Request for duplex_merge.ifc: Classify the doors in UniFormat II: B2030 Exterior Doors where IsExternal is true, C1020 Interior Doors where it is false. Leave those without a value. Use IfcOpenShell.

First a look at what the model holds.

```python
import ifcopenshell
import ifcopenshell.util.element

model = ifcopenshell.open("duplex_merge.ifc")
print(model.schema)
print("classifications:", [c.Name for c in model.by_type("IfcClassification")])
values = [ifcopenshell.util.element.get_pset(e, "Pset_DoorCommon", "IsExternal") for e in model.by_type("IfcDoor")]
for value in (True, False, None):
    print("IsExternal", value, values.count(value))
```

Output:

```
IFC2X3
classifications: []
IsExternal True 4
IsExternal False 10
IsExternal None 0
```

```python
import ifcopenshell
import ifcopenshell.api.classification
import ifcopenshell.util.element

model = ifcopenshell.open("duplex_merge.ifc")

# IFC2X3 requires Source and Edition and has no link from the project to the system.
system = model.create_entity("IfcClassification", Source="ASTM", Edition="E1557", Name="UniFormat II")

doors = model.by_type("IfcDoor")
external = {e: ifcopenshell.util.element.get_pset(e, "Pset_DoorCommon", "IsExternal") for e in doors}
for flag, code, name in ((True, "B2030", "Exterior Doors"), (False, "C1020", "Interior Doors")):
    products = [e for e in doors if external[e] is flag]
    ifcopenshell.api.classification.add_reference(
        model, products=products, classification=system, identification=code, name=name
    )
    print(code, len(products))

model.write("duplex_merge_v2.ifc")
```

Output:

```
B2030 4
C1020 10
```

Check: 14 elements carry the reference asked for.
